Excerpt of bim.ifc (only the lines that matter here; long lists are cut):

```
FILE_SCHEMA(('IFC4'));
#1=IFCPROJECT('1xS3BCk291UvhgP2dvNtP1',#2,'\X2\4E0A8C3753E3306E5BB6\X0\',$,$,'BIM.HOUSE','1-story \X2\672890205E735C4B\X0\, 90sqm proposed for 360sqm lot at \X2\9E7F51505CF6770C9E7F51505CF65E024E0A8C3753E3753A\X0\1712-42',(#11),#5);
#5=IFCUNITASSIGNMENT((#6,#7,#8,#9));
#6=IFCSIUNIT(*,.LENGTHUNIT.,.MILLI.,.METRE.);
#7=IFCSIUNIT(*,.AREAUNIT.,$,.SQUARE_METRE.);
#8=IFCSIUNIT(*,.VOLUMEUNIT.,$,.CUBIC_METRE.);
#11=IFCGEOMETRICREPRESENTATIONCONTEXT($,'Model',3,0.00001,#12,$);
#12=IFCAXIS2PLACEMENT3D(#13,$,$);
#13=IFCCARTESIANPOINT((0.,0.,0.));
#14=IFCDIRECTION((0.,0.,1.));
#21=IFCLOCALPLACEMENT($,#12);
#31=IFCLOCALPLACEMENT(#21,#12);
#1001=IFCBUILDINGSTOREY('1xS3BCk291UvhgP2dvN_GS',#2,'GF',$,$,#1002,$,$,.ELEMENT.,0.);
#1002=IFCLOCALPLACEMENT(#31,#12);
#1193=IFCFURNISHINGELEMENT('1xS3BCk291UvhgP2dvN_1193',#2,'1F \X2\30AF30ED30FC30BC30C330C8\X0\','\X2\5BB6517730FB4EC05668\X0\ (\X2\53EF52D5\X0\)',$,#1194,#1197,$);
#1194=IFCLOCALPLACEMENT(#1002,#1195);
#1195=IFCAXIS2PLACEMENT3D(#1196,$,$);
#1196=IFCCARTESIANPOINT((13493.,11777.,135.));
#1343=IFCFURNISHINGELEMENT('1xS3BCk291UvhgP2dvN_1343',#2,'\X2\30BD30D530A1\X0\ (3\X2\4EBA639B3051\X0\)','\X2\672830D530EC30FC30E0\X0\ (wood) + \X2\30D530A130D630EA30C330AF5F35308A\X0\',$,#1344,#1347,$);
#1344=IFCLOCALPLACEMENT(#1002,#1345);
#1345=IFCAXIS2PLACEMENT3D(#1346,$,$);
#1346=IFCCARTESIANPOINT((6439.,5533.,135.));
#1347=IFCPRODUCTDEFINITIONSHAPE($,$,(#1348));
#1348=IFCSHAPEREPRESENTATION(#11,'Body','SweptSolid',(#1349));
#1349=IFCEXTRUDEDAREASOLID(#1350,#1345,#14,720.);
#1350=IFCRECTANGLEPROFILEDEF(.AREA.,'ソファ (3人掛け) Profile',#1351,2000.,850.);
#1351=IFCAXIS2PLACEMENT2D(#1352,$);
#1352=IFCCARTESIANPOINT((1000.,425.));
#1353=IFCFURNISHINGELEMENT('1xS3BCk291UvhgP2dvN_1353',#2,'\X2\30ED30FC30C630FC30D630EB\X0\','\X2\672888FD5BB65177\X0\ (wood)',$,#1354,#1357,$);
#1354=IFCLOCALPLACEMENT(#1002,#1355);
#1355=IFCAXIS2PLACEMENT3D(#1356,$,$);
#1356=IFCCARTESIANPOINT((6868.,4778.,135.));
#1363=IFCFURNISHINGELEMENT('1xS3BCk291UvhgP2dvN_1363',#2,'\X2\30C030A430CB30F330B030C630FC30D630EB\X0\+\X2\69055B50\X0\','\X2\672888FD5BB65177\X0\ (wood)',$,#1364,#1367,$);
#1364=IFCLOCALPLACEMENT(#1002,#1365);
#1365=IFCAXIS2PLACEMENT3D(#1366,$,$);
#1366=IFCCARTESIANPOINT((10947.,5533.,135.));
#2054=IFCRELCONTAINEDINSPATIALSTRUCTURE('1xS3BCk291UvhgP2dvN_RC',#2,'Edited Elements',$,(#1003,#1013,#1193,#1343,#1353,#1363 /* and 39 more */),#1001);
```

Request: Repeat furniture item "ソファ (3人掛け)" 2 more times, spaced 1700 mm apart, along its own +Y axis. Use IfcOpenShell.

```python
import ifcopenshell
import ifcopenshell.api.geometry
import ifcopenshell.api.root
import ifcopenshell.util.element
import ifcopenshell.util.placement

model = ifcopenshell.open("bim.ifc")


def reuse_history(source, copy):
    """copy_class also copies each property set's owner history, people and application; keep the originals."""
    for rel in copy.IsDefinedBy:
        if rel.is_a("IfcRelDefinesByProperties") and (history := rel.RelatingPropertyDefinition.OwnerHistory):
            rel.RelatingPropertyDefinition.OwnerHistory = source.OwnerHistory
            ifcopenshell.util.element.remove_deep2(model, history)


source = model.by_guid("1xS3BCk291UvhgP2dvN_1343")
base = ifcopenshell.util.placement.get_local_placement(source.ObjectPlacement)
step = base[:3, 1] * 1700.0

for i in range(1, 3):
    copy = ifcopenshell.api.root.copy_class(model, product=source)
    copy.Representation = ifcopenshell.util.element.copy_deep(
        model, source.Representation, exclude=["IfcGeometricRepresentationContext", "IfcRepresentationMap"]
    )
    reuse_history(source, copy)
    matrix = base.copy()
    matrix[:3, 3] += i * step
    print("added at", matrix[:3, 3].round(3) + 0.0)
    ifcopenshell.api.geometry.edit_object_placement(model, product=copy, matrix=matrix, is_si=False)

model.write("bim-out.ifc")
```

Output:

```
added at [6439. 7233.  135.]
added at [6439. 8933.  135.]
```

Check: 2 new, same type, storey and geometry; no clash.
